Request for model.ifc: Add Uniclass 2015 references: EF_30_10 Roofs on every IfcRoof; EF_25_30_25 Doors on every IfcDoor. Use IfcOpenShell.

First a look at what the model holds.

```python
import ifcopenshell

model = ifcopenshell.open("model.ifc")
print(model.schema)
print("classifications:", [c.Name for c in model.by_type("IfcClassification")])
for ifc_class in ("IfcDoor", "IfcRoof", "IfcStair", "IfcWall", "IfcWindow"):
    print(ifc_class, len(model.by_type(ifc_class)))
```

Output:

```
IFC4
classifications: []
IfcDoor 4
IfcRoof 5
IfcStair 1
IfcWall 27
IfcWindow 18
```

```python
import ifcopenshell
import ifcopenshell.api.classification

model = ifcopenshell.open("model.ifc")

system = ifcopenshell.api.classification.add_classification(model, classification="Uniclass 2015")

codes = {
    "IfcRoof": ("EF_30_10", "Roofs"),
    "IfcDoor": ("EF_25_30_25", "Doors"),
}
for ifc_class, (code, name) in codes.items():
    products = model.by_type(ifc_class)
    ifcopenshell.api.classification.add_reference(
        model, products=products, classification=system, identification=code, name=name
    )
    print(code, len(products))

model.write("model-out.ifc")
```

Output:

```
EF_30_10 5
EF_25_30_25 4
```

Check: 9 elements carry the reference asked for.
